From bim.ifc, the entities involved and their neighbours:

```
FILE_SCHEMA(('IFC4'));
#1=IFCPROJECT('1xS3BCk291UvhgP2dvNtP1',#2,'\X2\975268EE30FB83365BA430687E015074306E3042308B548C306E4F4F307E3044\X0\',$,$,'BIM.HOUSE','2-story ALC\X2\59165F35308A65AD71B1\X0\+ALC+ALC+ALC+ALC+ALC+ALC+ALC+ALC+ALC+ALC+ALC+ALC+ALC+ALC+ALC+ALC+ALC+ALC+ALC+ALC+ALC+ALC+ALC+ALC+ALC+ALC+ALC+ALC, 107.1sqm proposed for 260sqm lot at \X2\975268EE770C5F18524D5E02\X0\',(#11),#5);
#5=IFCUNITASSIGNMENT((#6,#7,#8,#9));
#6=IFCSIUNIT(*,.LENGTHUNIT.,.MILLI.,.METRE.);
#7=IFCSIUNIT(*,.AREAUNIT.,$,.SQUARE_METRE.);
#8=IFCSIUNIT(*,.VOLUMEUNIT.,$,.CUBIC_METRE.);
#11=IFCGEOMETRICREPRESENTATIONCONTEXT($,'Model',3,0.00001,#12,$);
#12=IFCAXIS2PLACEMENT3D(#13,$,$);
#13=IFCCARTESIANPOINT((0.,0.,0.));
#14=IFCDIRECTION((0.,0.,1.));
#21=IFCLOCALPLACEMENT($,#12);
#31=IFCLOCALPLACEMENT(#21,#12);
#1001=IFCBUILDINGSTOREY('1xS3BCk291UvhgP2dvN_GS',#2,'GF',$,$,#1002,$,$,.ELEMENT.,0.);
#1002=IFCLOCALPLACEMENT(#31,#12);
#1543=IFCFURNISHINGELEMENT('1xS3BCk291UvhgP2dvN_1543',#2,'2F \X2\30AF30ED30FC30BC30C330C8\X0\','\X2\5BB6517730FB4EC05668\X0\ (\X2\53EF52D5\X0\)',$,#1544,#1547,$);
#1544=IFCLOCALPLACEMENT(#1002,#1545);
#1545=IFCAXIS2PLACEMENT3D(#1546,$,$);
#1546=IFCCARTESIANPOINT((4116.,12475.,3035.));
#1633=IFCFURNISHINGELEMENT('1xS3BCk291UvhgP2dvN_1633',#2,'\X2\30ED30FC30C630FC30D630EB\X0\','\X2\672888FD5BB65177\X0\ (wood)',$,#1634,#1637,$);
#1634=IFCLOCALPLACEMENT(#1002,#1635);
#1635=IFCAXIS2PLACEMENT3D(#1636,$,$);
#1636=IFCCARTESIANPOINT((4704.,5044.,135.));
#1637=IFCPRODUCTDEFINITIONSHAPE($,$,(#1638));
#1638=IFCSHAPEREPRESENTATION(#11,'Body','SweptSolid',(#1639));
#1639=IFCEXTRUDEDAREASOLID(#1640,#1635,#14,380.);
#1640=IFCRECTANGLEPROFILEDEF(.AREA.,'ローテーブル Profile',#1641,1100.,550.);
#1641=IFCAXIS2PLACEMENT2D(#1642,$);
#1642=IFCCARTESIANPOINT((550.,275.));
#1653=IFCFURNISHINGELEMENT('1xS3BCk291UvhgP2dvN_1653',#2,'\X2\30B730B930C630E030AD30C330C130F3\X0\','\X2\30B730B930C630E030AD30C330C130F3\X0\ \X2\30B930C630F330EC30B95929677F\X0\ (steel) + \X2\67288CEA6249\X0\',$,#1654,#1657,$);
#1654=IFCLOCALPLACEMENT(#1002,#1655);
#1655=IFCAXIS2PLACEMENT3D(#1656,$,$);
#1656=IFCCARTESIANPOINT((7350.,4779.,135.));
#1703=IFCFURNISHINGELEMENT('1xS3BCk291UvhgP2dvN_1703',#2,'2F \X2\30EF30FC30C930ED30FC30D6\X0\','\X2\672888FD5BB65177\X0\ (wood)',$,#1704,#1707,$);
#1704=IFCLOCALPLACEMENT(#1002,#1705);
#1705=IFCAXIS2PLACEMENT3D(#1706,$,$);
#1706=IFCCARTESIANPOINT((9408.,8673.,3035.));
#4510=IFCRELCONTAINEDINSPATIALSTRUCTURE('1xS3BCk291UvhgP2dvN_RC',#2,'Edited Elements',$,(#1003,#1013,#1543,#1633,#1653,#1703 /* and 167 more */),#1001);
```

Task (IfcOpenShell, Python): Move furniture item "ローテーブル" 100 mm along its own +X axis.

```python
import ifcopenshell
import ifcopenshell.api.geometry
import ifcopenshell.util.placement
import ifcopenshell.util.unit

model = ifcopenshell.open("bim.ifc")
unit_scale = ifcopenshell.util.unit.calculate_unit_scale(model)

item = model.by_guid("1xS3BCk291UvhgP2dvN_1633")
matrix = ifcopenshell.util.placement.get_local_placement(item.ObjectPlacement)
matrix[:3, 3] += matrix[:3, 0] * 0.1 / unit_scale
ifcopenshell.api.geometry.edit_object_placement(model, product=item, matrix=matrix, is_si=False)

print(ifcopenshell.util.placement.get_local_placement(item.ObjectPlacement).round(3) + 0.0)

model.write("bim_rev.ifc")
```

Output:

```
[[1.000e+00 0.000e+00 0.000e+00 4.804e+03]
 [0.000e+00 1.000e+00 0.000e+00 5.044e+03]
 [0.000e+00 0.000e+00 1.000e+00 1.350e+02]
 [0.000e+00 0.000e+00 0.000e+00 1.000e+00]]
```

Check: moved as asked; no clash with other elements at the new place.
